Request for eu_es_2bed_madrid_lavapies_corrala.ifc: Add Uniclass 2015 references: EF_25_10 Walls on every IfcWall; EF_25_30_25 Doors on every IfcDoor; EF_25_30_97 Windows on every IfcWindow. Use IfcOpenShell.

First a look at what the model holds.

```python
import ifcopenshell

model = ifcopenshell.open("eu_es_2bed_madrid_lavapies_corrala.ifc")
print(model.schema)
print("classifications:", [c.Name for c in model.by_type("IfcClassification")])
for ifc_class in ("IfcDoor", "IfcRoof", "IfcStair", "IfcWall", "IfcWindow"):
    print(ifc_class, len(model.by_type(ifc_class)))
```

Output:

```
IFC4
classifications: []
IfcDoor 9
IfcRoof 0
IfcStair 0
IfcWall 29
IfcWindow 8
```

```python
import ifcopenshell
import ifcopenshell.api.classification

model = ifcopenshell.open("eu_es_2bed_madrid_lavapies_corrala.ifc")

system = ifcopenshell.api.classification.add_classification(model, classification="Uniclass 2015")

codes = {
    "IfcWall": ("EF_25_10", "Walls"),
    "IfcDoor": ("EF_25_30_25", "Doors"),
    "IfcWindow": ("EF_25_30_97", "Windows"),
}
for ifc_class, (code, name) in codes.items():
    products = model.by_type(ifc_class)
    ifcopenshell.api.classification.add_reference(
        model, products=products, classification=system, identification=code, name=name
    )
    print(code, len(products))

model.write("eu_es_2bed_madrid_lavapies_corrala_rev.ifc")
```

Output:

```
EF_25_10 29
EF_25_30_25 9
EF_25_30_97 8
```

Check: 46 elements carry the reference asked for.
